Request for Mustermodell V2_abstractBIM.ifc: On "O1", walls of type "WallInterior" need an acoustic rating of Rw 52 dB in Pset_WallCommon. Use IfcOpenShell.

First a look at what the model holds.

```python
import ifcopenshell
import ifcopenshell.util.element

model = ifcopenshell.open("Mustermodell V2_abstractBIM.ifc")
print(model.schema)
storey = next(s for s in model.by_type("IfcBuildingStorey") if s.Name == "O1")
walls = [e for e in ifcopenshell.util.element.get_decomposition(storey) if e.is_a("IfcWall")]
seen = {}
for e in walls:
    element_type = ifcopenshell.util.element.get_type(e)
    key = (element_type.Name if element_type != e and element_type else None, ifcopenshell.util.element.get_pset(e, "Pset_WallCommon", "AcousticRating"))
    seen[key] = seen.get(key, 0) + 1
for (name, value), count in sorted(seen.items(), key=str):
    print(count, "x", name, "|", value)
```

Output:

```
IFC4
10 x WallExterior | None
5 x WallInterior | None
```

```python
import ifcopenshell
import ifcopenshell.api.pset
import ifcopenshell.util.element

model = ifcopenshell.open("Mustermodell V2_abstractBIM.ifc")

storey = next(s for s in model.by_type("IfcBuildingStorey") if s.Name == "O1")
walls = [e for e in ifcopenshell.util.element.get_decomposition(storey) if e.is_a("IfcWall")]

count = 0
for e in walls:
    element_type = ifcopenshell.util.element.get_type(e)
    if element_type in (None, e) or element_type.Name != "WallInterior":
        continue
    # add_pset returns the element's existing set when there is one.
    pset = ifcopenshell.api.pset.add_pset(model, product=e, name="Pset_WallCommon")
    ifcopenshell.api.pset.edit_pset(model, pset=pset, properties={"AcousticRating": "Rw 52 dB"})
    count += 1

print(count, "walls updated")

model.write("Mustermodell V2_abstractBIM_edited.ifc")
```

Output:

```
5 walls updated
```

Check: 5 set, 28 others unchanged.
